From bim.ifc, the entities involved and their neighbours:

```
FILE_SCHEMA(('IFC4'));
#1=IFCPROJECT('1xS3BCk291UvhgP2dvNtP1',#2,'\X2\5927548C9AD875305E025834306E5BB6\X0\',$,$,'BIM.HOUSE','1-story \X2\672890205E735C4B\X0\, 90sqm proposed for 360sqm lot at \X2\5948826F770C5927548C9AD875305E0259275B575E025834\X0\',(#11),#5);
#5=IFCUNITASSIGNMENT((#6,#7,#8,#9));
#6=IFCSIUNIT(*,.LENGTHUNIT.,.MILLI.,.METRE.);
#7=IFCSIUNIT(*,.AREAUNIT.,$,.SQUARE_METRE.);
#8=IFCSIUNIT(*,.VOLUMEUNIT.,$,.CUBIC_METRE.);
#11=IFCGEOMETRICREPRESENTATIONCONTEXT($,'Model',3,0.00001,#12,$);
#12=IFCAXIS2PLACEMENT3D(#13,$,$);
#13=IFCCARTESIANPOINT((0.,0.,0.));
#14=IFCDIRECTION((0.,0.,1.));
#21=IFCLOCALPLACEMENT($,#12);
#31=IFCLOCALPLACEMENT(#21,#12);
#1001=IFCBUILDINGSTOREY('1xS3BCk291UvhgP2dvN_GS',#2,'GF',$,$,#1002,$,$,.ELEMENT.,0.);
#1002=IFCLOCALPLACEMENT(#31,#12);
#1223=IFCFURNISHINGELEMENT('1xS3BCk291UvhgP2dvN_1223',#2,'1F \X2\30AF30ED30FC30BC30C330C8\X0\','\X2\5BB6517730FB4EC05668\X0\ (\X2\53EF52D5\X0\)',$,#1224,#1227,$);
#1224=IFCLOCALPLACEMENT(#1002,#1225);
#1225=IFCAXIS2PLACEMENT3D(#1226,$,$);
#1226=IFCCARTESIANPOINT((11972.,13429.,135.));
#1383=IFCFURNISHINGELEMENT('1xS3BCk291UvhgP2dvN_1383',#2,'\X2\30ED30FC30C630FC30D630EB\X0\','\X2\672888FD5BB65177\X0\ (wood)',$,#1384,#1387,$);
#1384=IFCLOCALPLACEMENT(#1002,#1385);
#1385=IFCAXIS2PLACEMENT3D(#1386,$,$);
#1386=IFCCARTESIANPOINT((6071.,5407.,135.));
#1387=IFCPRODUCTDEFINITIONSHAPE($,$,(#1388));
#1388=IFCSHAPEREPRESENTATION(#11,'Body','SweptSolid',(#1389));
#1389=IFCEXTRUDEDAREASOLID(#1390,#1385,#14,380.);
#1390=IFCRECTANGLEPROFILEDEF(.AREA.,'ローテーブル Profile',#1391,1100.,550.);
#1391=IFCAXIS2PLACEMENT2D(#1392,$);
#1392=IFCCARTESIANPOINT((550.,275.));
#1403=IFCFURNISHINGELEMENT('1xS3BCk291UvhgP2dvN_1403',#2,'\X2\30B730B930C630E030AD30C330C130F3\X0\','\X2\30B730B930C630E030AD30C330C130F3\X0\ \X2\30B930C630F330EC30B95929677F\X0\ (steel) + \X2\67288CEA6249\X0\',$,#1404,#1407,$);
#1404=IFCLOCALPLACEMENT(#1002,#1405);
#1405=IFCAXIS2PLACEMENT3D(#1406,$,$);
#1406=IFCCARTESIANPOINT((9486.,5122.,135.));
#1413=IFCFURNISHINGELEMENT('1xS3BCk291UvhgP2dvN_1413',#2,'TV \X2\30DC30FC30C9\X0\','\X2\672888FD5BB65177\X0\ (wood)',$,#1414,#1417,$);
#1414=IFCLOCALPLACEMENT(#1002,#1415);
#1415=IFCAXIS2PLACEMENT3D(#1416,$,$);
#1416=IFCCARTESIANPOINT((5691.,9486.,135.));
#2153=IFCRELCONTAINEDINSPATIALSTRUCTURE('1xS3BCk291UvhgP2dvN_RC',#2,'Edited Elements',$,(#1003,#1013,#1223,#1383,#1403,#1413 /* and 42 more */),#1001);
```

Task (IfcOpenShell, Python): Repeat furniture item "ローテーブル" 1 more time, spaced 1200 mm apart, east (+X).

```python
import numpy as np
import ifcopenshell
import ifcopenshell.api.geometry
import ifcopenshell.api.root
import ifcopenshell.util.element
import ifcopenshell.util.placement

model = ifcopenshell.open("bim.ifc")


def reuse_history(source, copy):
    """copy_class also copies each property set's owner history, people and application; keep the originals."""
    for rel in copy.IsDefinedBy:
        if rel.is_a("IfcRelDefinesByProperties") and (history := rel.RelatingPropertyDefinition.OwnerHistory):
            rel.RelatingPropertyDefinition.OwnerHistory = source.OwnerHistory
            ifcopenshell.util.element.remove_deep2(model, history)


source = model.by_guid("1xS3BCk291UvhgP2dvN_1383")
base = ifcopenshell.util.placement.get_local_placement(source.ObjectPlacement)
step = np.array([1.0, 0.0, 0.0]) * 1200.0

for i in range(1, 2):
    copy = ifcopenshell.api.root.copy_class(model, product=source)
    copy.Representation = ifcopenshell.util.element.copy_deep(
        model, source.Representation, exclude=["IfcGeometricRepresentationContext", "IfcRepresentationMap"]
    )
    reuse_history(source, copy)
    matrix = base.copy()
    matrix[:3, 3] += i * step
    print("added at", matrix[:3, 3].round(3) + 0.0)
    ifcopenshell.api.geometry.edit_object_placement(model, product=copy, matrix=matrix, is_si=False)

model.write("bim-out.ifc")
```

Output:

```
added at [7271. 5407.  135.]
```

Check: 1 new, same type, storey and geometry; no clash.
